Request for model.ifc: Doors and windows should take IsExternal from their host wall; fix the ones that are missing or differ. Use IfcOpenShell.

First a look at what the model holds.

```python
import ifcopenshell
import ifcopenshell.util.element

model = ifcopenshell.open("model.ifc")
print(model.schema)
seen = {}
for e in model.by_type("IfcDoor") + model.by_type("IfcWindow"):
    if not e.FillsVoids:
        continue
    host = e.FillsVoids[0].RelatingOpeningElement.VoidsElements[0].RelatingBuildingElement
    own = ifcopenshell.util.element.get_pset(e, f"Pset_{e.is_a()[3:].removesuffix('StandardCase')}Common", "IsExternal")
    wall = ifcopenshell.util.element.get_pset(host, "Pset_WallCommon", "IsExternal")
    seen[e.is_a(), own, wall] = seen.get((e.is_a(), own, wall), 0) + 1
for (cls, own, wall), count in sorted(seen.items(), key=str):
    print(count, cls, "IsExternal:", own, "| host wall:", wall)
```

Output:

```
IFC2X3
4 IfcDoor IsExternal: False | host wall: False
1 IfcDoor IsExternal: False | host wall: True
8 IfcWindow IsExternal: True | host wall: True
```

```python
import ifcopenshell
import ifcopenshell.api.pset
import ifcopenshell.util.element

model = ifcopenshell.open("model.ifc")

count = 0
for ifc_class, pset_name in (("IfcDoor", "Pset_DoorCommon"), ("IfcWindow", "Pset_WindowCommon")):
    for e in model.by_type(ifc_class):
        if not e.FillsVoids:
            continue
        host = e.FillsVoids[0].RelatingOpeningElement.VoidsElements[0].RelatingBuildingElement
        external = ifcopenshell.util.element.get_pset(host, "Pset_WallCommon", "IsExternal")
        if external is None or ifcopenshell.util.element.get_pset(e, pset_name, "IsExternal") == external:
            continue
        pset = ifcopenshell.api.pset.add_pset(model, product=e, name=pset_name)
        ifcopenshell.api.pset.edit_pset(model, pset=pset, properties={"IsExternal": external})
        count += 1

print(count, "updated")

model.write("model_rev.ifc")
```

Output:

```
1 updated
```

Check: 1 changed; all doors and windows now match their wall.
